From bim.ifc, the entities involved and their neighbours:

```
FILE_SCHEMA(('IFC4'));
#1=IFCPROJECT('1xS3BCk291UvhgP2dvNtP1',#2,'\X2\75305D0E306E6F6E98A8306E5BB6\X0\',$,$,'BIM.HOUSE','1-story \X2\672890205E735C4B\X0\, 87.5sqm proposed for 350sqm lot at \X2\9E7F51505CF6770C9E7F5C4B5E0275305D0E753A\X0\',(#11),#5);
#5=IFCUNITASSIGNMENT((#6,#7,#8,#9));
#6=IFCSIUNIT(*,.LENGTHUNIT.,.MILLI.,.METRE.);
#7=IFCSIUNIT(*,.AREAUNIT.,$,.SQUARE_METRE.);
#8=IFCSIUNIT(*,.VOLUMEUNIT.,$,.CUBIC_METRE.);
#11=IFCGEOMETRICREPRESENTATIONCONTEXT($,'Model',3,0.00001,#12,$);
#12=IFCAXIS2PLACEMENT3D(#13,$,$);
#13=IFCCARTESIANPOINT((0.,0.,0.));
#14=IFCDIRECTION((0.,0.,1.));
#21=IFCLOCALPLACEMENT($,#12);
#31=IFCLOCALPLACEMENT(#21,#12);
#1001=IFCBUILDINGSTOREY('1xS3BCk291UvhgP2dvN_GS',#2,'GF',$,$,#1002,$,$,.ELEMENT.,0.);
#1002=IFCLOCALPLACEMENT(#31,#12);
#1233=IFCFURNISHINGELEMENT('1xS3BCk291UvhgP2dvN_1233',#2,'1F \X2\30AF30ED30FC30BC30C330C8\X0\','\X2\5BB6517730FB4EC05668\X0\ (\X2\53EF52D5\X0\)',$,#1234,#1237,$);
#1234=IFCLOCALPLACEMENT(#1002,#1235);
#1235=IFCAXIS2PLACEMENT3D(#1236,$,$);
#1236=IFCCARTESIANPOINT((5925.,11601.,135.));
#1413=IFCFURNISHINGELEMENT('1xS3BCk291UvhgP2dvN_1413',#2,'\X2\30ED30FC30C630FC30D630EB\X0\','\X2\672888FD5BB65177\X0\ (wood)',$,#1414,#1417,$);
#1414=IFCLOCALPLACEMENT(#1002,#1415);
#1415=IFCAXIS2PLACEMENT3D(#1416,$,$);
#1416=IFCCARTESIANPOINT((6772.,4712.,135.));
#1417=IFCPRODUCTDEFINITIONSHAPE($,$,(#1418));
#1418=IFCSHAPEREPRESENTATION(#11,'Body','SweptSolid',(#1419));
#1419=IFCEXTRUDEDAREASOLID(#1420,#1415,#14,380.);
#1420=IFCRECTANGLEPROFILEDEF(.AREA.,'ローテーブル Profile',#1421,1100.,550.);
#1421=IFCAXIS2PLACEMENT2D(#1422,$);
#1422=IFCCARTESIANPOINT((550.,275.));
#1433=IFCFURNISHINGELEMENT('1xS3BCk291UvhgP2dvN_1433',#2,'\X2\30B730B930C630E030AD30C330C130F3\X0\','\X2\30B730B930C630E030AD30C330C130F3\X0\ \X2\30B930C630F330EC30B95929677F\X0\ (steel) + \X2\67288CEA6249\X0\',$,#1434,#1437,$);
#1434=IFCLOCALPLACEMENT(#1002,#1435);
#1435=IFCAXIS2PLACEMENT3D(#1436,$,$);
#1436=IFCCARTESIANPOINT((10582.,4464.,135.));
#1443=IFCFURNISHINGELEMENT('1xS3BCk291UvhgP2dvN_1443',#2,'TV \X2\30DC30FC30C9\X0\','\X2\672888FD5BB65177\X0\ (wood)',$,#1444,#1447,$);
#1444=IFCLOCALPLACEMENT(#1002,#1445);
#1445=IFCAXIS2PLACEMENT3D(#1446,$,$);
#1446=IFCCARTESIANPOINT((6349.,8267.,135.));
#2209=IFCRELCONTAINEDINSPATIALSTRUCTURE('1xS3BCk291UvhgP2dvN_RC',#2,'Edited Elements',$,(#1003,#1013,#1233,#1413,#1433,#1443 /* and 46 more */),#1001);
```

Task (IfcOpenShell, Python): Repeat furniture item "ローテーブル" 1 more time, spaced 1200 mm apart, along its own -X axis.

```python
import ifcopenshell
import ifcopenshell.api.geometry
import ifcopenshell.api.root
import ifcopenshell.util.element
import ifcopenshell.util.placement
import ifcopenshell.util.unit

model = ifcopenshell.open("bim.ifc")
unit_scale = ifcopenshell.util.unit.calculate_unit_scale(model)


def reuse_history(source, copy):
    """copy_class also copies each property set's owner history, people and application; keep the originals."""
    for rel in copy.IsDefinedBy:
        if rel.is_a("IfcRelDefinesByProperties") and (history := rel.RelatingPropertyDefinition.OwnerHistory):
            rel.RelatingPropertyDefinition.OwnerHistory = source.OwnerHistory
            ifcopenshell.util.element.remove_deep2(model, history)


source = model.by_guid("1xS3BCk291UvhgP2dvN_1413")
base = ifcopenshell.util.placement.get_local_placement(source.ObjectPlacement)
step = -base[:3, 0] * 1.2 / unit_scale

for i in range(1, 2):
    copy = ifcopenshell.api.root.copy_class(model, product=source)
    copy.Representation = ifcopenshell.util.element.copy_deep(
        model, source.Representation, exclude=["IfcGeometricRepresentationContext", "IfcRepresentationMap"]
    )
    reuse_history(source, copy)
    matrix = base.copy()
    matrix[:3, 3] += i * step
    print("added at", matrix[:3, 3].round(3) + 0.0)
    ifcopenshell.api.geometry.edit_object_placement(model, product=copy, matrix=matrix, is_si=False)

model.write("bim_edited.ifc")
```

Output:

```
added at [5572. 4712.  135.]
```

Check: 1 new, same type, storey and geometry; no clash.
